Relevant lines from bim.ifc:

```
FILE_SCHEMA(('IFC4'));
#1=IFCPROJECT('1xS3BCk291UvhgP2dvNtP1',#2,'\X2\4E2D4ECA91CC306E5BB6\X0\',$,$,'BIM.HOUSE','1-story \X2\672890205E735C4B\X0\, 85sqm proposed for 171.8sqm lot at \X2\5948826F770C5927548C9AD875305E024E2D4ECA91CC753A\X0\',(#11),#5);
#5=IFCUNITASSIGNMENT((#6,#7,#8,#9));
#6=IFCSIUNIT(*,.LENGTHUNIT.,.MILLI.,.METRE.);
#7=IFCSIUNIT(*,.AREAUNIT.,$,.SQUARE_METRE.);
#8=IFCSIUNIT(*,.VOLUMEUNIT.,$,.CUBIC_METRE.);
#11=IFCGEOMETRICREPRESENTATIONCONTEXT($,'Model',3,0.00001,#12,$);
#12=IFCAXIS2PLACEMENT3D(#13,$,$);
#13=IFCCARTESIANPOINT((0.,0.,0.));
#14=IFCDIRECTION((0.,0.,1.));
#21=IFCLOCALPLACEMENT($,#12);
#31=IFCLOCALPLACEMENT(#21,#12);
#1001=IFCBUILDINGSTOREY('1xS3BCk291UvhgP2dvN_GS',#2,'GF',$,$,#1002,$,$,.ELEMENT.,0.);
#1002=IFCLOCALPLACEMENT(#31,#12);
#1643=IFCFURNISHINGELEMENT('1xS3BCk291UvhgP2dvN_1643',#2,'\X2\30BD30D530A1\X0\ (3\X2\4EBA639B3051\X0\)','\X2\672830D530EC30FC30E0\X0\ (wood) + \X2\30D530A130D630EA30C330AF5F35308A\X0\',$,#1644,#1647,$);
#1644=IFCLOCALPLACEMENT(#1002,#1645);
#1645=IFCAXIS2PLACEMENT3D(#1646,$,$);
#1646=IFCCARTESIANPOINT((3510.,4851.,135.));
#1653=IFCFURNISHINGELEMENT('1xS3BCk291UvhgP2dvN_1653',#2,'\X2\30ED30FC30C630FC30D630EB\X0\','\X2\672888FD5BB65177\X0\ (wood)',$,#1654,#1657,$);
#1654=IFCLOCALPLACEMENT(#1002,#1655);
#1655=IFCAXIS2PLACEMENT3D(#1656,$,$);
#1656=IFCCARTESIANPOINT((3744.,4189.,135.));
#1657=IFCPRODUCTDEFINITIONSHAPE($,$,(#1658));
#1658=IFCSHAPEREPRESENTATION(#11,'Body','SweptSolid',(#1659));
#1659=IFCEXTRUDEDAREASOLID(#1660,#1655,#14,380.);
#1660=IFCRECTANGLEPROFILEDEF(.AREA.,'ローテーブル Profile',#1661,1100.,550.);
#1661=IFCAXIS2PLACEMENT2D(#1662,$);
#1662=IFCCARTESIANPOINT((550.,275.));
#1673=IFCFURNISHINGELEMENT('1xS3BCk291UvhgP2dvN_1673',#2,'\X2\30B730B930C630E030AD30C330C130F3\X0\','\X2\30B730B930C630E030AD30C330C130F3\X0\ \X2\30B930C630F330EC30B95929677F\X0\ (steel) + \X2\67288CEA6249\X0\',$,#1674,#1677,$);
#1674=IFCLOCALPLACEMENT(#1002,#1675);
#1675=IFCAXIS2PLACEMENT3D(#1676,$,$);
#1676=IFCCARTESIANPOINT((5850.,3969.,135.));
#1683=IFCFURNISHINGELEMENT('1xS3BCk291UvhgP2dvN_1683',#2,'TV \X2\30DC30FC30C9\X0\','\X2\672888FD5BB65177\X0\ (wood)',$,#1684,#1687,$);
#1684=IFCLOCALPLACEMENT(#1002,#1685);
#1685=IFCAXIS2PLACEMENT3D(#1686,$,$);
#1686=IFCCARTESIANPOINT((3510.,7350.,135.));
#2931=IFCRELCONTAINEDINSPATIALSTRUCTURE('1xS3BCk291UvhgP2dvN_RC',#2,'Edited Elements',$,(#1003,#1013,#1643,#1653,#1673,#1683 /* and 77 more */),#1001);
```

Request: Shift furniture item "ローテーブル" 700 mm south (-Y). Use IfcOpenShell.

```python
import ifcopenshell
import ifcopenshell.api.geometry
import ifcopenshell.util.placement

model = ifcopenshell.open("bim.ifc")

item = model.by_guid("1xS3BCk291UvhgP2dvN_1653")
matrix = ifcopenshell.util.placement.get_local_placement(item.ObjectPlacement)
matrix[1, 3] -= 700.0
ifcopenshell.api.geometry.edit_object_placement(model, product=item, matrix=matrix, is_si=False)

print(ifcopenshell.util.placement.get_local_placement(item.ObjectPlacement).round(3) + 0.0)

model.write("bim_rev.ifc")
```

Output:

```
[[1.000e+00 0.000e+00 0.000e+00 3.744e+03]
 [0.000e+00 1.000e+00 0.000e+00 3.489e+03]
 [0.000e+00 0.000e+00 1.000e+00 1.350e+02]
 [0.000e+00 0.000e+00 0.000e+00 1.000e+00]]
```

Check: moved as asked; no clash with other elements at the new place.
